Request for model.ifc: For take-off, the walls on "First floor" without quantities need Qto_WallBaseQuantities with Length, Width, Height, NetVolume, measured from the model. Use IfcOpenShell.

First a look at what the model holds.

```python
import ifcopenshell
import ifcopenshell.util.element
import ifcopenshell.util.unit

model = ifcopenshell.open("model.ifc")
print(model.schema)
for unit_type in ("LENGTHUNIT", "AREAUNIT", "VOLUMEUNIT"):
    print(unit_type, ifcopenshell.util.unit.calculate_unit_scale(model, unit_type))
storey = next(s for s in model.by_type("IfcBuildingStorey") if s.Name == "First floor")
walls = [e for e in ifcopenshell.util.element.get_decomposition(storey) if e.is_a("IfcWall")]
for e in sorted(walls, key=lambda e: e.id()):
    print(e.id(), e.is_a(), e.Name, list(ifcopenshell.util.element.get_psets(e, qtos_only=True)), sep=" | ")
```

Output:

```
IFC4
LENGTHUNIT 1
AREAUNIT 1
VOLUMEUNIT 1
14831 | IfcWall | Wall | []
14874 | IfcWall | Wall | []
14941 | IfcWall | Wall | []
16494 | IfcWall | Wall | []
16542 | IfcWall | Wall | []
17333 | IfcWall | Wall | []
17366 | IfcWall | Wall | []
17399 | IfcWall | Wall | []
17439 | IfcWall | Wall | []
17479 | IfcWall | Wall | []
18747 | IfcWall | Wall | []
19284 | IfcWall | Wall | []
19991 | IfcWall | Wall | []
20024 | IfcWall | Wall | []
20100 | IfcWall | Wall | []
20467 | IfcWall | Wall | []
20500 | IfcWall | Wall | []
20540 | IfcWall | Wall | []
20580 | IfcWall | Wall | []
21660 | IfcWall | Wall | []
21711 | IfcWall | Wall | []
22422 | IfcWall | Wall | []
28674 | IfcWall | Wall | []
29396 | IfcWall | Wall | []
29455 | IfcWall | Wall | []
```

```python
import ifcopenshell
import ifcopenshell.api.pset
import ifcopenshell.geom
import ifcopenshell.util.element
import ifcopenshell.util.shape
import ifcopenshell.util.unit

model = ifcopenshell.open("model.ifc")
unit_scale = ifcopenshell.util.unit.calculate_unit_scale(model)
volume_scale = ifcopenshell.util.unit.calculate_unit_scale(model, "VOLUMEUNIT")
settings = ifcopenshell.geom.settings()

storey = next(s for s in model.by_type("IfcBuildingStorey") if s.Name == "First floor")
walls = [e for e in ifcopenshell.util.element.get_decomposition(storey) if e.is_a("IfcWall")]

for e in sorted(walls, key=lambda e: e.id()):
    if ifcopenshell.util.element.get_psets(e, qtos_only=True, should_inherit=False):
        continue
    # Geometry comes back in metres, in the element's own axes.
    shape = ifcopenshell.geom.create_shape(settings, e)
    values = {
        "Length": ifcopenshell.util.shape.get_x(shape.geometry) / unit_scale,
        "Width": ifcopenshell.util.shape.get_y(shape.geometry) / unit_scale,
        "Height": ifcopenshell.util.shape.get_z(shape.geometry) / unit_scale,
        "NetVolume": ifcopenshell.util.shape.get_volume(shape.geometry) / volume_scale,
    }
    qto = ifcopenshell.api.pset.add_qto(model, product=e, name="Qto_WallBaseQuantities")
    ifcopenshell.api.pset.edit_qto(model, qto=qto, properties=values)
    print(e.id(), {k: round(v, 3) for k, v in values.items()})

model.write("model-out.ifc")
```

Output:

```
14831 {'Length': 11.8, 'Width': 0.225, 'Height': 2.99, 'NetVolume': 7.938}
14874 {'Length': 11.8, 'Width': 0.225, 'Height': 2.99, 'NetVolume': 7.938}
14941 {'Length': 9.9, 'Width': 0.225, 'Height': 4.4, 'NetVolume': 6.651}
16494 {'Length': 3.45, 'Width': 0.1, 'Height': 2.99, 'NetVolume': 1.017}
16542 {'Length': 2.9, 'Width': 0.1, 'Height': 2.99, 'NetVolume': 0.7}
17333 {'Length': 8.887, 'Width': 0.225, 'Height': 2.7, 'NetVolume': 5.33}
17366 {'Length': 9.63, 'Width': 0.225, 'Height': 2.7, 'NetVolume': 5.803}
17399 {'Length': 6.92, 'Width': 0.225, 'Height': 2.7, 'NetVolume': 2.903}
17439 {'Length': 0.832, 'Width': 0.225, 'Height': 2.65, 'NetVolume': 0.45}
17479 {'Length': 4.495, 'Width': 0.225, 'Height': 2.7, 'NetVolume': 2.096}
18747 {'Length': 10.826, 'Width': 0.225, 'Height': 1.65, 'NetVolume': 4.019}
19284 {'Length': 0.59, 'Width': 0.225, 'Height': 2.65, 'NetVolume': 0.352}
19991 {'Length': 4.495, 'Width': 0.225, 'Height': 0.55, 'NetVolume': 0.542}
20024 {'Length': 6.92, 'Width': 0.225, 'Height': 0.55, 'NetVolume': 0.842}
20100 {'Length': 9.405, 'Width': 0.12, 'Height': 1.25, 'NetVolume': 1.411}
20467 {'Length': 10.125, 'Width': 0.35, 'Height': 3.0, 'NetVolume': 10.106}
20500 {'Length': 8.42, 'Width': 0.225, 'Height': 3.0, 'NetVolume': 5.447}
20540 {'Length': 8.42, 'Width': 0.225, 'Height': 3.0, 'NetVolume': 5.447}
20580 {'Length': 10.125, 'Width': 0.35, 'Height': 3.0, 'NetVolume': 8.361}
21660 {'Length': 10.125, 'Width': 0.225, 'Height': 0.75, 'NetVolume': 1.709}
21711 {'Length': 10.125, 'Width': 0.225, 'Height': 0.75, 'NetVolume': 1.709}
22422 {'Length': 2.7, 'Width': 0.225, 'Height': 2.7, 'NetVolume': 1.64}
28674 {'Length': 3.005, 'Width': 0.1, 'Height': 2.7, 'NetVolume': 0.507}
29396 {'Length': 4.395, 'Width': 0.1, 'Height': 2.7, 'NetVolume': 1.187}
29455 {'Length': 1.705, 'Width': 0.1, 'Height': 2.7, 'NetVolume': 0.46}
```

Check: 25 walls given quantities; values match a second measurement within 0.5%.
